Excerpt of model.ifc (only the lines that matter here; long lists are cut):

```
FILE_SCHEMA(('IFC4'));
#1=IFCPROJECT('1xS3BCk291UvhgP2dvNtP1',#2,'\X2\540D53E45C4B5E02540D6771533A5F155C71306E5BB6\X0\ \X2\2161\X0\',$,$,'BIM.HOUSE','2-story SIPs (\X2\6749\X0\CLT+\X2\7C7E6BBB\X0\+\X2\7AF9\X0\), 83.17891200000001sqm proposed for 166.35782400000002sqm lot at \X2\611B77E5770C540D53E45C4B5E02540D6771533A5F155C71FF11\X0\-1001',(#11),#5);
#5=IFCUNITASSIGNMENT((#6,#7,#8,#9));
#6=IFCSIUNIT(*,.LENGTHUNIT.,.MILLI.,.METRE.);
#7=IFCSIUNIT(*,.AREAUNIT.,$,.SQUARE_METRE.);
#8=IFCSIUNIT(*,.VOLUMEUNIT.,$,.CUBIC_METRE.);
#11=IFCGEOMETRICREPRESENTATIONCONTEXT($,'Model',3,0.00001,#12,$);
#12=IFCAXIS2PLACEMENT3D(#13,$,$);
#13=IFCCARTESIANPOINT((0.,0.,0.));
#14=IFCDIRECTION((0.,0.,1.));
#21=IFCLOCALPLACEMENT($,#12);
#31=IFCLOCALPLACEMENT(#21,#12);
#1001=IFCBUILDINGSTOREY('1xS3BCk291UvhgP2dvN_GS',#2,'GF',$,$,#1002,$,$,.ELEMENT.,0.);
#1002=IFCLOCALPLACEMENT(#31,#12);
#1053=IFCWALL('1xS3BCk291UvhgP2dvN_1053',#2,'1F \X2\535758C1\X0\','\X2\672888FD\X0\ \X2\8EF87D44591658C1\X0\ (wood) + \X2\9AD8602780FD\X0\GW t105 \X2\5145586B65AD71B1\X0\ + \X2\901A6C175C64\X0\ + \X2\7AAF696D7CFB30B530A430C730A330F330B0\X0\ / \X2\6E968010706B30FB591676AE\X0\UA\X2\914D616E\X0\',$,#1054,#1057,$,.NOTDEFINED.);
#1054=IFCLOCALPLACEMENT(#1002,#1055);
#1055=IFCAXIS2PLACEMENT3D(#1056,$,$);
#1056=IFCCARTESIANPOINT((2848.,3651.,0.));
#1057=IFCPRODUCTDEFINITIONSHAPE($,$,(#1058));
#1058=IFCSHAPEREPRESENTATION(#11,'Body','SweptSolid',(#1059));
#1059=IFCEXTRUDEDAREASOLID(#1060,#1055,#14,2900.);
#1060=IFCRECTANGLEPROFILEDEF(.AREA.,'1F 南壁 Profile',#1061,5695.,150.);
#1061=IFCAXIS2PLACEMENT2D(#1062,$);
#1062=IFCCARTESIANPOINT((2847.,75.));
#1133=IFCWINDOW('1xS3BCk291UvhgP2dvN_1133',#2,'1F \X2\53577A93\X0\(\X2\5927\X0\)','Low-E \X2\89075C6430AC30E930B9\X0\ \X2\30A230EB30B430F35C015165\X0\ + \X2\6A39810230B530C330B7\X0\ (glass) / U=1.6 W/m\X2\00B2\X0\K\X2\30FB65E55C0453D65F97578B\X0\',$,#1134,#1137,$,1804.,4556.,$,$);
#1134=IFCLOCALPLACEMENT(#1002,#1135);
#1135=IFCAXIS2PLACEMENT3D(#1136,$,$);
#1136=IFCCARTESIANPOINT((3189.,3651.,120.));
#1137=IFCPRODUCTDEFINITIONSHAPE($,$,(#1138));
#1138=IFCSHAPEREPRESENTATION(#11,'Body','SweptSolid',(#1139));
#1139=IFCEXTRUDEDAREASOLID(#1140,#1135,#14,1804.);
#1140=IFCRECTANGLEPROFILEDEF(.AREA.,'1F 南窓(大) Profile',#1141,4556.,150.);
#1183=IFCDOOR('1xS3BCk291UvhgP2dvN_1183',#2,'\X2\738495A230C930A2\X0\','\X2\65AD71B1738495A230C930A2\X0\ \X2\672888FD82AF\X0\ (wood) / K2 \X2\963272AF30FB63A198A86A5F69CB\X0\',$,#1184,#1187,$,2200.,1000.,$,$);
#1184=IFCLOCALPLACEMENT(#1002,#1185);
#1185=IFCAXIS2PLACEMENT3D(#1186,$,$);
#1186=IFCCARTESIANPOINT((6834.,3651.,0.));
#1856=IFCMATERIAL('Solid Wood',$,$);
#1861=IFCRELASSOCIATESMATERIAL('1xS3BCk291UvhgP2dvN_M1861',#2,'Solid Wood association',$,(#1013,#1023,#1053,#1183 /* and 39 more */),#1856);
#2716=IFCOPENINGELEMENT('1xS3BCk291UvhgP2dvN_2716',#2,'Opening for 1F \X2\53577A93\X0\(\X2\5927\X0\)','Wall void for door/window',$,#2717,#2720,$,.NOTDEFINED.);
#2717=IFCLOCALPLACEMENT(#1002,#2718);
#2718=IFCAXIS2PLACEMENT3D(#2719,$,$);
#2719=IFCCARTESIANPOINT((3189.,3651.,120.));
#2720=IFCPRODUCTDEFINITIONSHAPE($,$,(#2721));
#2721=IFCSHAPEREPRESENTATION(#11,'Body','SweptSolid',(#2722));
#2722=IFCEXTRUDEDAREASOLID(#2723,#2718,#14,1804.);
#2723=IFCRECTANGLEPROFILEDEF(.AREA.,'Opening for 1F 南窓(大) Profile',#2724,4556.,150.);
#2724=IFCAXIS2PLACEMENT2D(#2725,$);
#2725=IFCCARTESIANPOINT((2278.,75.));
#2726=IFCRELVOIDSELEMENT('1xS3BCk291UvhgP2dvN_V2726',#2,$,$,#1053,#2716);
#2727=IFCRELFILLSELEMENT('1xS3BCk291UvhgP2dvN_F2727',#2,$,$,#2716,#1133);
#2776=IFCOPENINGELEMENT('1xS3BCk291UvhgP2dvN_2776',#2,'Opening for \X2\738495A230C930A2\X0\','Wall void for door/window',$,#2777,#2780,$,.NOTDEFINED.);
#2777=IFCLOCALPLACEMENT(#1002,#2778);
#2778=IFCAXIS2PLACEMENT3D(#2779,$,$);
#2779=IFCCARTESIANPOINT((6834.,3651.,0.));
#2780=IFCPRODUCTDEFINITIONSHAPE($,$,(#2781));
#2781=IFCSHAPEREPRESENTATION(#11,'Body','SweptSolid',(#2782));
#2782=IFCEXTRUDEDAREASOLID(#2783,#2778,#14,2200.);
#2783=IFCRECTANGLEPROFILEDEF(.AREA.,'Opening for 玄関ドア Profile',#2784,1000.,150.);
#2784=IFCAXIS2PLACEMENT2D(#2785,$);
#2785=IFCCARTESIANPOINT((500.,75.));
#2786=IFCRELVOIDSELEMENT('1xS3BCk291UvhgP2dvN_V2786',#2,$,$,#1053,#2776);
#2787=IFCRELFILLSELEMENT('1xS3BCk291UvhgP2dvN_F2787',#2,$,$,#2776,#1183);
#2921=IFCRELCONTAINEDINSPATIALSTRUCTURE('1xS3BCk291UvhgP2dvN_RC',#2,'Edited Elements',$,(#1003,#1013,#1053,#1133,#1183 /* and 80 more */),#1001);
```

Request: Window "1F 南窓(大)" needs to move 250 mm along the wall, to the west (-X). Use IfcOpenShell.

```python
import ifcopenshell
import ifcopenshell.api.geometry
import ifcopenshell.util.placement
import ifcopenshell.util.unit

model = ifcopenshell.open("model.ifc")
unit_scale = ifcopenshell.util.unit.calculate_unit_scale(model)

window = model.by_guid("1xS3BCk291UvhgP2dvN_1133")
opening = window.FillsVoids[0].RelatingOpeningElement
wall = opening.VoidsElements[0].RelatingBuildingElement

wall_matrix = ifcopenshell.util.placement.get_local_placement(wall.ObjectPlacement)
shift = wall_matrix[:3, 0] * -0.25 / unit_scale
before = ifcopenshell.util.placement.get_local_placement(window.ObjectPlacement)[:3, 3].copy()

# The window is not placed relative to its opening, so move both.
for product in (opening, window):
    matrix = ifcopenshell.util.placement.get_local_placement(product.ObjectPlacement)
    matrix[:3, 3] += shift
    ifcopenshell.api.geometry.edit_object_placement(model, product=product, matrix=matrix, is_si=False)

after = ifcopenshell.util.placement.get_local_placement(window.ObjectPlacement)[:3, 3]
print("window moved by", (after - before).round(3) + 0.0)

model.write("model_edited.ifc")
```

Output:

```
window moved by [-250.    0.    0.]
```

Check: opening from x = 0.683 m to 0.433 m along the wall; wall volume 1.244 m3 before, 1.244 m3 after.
